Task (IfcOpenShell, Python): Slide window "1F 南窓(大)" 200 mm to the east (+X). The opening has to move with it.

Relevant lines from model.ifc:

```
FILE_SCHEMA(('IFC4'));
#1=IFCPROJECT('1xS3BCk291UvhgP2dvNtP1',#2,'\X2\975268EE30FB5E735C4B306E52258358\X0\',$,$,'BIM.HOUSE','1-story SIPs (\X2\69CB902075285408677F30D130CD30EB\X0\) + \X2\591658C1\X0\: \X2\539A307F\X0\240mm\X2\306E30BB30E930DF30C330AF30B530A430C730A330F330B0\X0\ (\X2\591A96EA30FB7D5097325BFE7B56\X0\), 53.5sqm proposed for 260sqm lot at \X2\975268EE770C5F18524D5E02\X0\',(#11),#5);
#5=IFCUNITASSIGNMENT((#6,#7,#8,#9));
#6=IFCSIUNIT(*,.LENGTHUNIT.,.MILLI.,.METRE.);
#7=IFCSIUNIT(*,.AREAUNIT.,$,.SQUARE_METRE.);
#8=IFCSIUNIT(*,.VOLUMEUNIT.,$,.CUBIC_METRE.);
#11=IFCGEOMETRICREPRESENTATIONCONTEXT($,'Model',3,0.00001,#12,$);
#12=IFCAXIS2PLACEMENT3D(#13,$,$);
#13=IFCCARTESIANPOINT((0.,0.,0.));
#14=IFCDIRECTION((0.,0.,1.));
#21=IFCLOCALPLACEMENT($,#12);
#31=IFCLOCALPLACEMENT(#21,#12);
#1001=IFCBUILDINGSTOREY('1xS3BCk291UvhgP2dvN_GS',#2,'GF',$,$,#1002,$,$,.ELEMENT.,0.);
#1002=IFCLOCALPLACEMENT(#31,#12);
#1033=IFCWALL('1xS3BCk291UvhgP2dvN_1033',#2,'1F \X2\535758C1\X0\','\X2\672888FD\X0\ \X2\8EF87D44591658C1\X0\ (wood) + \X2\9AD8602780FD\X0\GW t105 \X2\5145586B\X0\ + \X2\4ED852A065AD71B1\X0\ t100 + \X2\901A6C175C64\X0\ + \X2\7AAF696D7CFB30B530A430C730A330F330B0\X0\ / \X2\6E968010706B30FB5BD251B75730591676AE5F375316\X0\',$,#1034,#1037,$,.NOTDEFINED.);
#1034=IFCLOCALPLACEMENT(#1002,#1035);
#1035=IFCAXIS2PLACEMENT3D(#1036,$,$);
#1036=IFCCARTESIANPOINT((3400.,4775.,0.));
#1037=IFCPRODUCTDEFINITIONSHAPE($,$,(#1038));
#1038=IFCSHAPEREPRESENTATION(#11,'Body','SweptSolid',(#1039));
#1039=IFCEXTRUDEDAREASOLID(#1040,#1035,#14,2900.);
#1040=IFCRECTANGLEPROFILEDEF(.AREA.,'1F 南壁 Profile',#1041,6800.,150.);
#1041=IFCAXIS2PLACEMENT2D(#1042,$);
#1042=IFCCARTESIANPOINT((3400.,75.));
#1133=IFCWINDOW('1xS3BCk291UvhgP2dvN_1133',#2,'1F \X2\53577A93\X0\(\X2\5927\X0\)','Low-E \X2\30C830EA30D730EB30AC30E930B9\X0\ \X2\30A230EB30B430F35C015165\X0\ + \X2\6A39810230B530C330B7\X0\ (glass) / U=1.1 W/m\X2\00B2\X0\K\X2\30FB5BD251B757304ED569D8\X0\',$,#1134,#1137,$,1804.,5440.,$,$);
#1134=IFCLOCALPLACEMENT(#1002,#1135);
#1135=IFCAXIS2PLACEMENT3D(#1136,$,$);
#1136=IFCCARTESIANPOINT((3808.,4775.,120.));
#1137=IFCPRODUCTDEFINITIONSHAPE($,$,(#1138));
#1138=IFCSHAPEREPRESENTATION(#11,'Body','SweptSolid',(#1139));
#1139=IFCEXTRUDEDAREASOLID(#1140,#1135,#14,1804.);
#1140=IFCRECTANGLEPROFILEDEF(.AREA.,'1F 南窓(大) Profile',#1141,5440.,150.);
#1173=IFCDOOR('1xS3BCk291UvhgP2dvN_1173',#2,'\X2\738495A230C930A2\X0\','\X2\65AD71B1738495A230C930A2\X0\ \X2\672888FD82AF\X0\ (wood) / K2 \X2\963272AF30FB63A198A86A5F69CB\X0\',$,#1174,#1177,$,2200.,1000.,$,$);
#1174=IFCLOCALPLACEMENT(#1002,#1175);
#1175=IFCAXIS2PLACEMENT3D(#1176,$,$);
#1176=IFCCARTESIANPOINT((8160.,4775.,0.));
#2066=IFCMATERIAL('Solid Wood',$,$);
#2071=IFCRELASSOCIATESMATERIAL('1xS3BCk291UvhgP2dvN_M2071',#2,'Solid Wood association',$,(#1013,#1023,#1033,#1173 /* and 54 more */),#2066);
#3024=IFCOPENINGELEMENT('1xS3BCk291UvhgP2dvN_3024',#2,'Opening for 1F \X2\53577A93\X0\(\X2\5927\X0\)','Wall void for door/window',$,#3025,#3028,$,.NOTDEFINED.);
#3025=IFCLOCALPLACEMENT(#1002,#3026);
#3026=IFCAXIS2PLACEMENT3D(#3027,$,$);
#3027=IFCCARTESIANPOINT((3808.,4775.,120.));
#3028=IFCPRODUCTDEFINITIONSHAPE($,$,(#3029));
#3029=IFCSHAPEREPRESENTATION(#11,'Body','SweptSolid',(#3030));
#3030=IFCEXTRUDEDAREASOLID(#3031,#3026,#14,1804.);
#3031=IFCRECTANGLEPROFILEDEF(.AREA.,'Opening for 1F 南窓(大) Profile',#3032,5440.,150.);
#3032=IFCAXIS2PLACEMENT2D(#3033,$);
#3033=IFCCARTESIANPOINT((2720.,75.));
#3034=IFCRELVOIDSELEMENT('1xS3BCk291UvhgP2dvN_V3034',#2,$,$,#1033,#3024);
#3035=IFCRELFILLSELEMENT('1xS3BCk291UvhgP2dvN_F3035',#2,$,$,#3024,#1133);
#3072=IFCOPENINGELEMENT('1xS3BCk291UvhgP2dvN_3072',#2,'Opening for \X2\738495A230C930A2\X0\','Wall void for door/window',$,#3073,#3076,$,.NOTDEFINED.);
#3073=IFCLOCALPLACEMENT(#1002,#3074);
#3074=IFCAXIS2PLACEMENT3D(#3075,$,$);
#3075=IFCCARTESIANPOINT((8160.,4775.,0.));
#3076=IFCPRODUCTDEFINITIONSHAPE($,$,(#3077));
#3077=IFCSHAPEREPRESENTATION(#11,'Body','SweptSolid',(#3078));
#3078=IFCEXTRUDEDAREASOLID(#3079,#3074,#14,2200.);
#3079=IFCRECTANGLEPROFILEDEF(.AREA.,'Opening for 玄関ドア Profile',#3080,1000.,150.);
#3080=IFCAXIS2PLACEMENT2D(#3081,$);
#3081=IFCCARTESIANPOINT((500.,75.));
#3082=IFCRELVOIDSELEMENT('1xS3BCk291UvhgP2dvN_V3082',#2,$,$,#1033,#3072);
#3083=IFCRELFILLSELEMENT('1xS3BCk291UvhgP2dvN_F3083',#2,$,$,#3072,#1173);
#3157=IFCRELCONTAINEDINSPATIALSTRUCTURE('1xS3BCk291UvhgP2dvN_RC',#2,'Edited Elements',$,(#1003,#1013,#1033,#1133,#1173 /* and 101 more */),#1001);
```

```python
import ifcopenshell
import ifcopenshell.api.geometry
import ifcopenshell.util.placement

model = ifcopenshell.open("model.ifc")

window = model.by_guid("1xS3BCk291UvhgP2dvN_1133")
opening = window.FillsVoids[0].RelatingOpeningElement
wall = opening.VoidsElements[0].RelatingBuildingElement

wall_matrix = ifcopenshell.util.placement.get_local_placement(wall.ObjectPlacement)
shift = wall_matrix[:3, 0] * 200.0
before = ifcopenshell.util.placement.get_local_placement(window.ObjectPlacement)[:3, 3].copy()

# The window is not placed relative to its opening, so move both.
for product in (opening, window):
    matrix = ifcopenshell.util.placement.get_local_placement(product.ObjectPlacement)
    matrix[:3, 3] += shift
    ifcopenshell.api.geometry.edit_object_placement(model, product=product, matrix=matrix, is_si=False)

after = ifcopenshell.util.placement.get_local_placement(window.ObjectPlacement)[:3, 3]
print("window moved by", (after - before).round(3) + 0.0)

model.write("model-out.ifc")
```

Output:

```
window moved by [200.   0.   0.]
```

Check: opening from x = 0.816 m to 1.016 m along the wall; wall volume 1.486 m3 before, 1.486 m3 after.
